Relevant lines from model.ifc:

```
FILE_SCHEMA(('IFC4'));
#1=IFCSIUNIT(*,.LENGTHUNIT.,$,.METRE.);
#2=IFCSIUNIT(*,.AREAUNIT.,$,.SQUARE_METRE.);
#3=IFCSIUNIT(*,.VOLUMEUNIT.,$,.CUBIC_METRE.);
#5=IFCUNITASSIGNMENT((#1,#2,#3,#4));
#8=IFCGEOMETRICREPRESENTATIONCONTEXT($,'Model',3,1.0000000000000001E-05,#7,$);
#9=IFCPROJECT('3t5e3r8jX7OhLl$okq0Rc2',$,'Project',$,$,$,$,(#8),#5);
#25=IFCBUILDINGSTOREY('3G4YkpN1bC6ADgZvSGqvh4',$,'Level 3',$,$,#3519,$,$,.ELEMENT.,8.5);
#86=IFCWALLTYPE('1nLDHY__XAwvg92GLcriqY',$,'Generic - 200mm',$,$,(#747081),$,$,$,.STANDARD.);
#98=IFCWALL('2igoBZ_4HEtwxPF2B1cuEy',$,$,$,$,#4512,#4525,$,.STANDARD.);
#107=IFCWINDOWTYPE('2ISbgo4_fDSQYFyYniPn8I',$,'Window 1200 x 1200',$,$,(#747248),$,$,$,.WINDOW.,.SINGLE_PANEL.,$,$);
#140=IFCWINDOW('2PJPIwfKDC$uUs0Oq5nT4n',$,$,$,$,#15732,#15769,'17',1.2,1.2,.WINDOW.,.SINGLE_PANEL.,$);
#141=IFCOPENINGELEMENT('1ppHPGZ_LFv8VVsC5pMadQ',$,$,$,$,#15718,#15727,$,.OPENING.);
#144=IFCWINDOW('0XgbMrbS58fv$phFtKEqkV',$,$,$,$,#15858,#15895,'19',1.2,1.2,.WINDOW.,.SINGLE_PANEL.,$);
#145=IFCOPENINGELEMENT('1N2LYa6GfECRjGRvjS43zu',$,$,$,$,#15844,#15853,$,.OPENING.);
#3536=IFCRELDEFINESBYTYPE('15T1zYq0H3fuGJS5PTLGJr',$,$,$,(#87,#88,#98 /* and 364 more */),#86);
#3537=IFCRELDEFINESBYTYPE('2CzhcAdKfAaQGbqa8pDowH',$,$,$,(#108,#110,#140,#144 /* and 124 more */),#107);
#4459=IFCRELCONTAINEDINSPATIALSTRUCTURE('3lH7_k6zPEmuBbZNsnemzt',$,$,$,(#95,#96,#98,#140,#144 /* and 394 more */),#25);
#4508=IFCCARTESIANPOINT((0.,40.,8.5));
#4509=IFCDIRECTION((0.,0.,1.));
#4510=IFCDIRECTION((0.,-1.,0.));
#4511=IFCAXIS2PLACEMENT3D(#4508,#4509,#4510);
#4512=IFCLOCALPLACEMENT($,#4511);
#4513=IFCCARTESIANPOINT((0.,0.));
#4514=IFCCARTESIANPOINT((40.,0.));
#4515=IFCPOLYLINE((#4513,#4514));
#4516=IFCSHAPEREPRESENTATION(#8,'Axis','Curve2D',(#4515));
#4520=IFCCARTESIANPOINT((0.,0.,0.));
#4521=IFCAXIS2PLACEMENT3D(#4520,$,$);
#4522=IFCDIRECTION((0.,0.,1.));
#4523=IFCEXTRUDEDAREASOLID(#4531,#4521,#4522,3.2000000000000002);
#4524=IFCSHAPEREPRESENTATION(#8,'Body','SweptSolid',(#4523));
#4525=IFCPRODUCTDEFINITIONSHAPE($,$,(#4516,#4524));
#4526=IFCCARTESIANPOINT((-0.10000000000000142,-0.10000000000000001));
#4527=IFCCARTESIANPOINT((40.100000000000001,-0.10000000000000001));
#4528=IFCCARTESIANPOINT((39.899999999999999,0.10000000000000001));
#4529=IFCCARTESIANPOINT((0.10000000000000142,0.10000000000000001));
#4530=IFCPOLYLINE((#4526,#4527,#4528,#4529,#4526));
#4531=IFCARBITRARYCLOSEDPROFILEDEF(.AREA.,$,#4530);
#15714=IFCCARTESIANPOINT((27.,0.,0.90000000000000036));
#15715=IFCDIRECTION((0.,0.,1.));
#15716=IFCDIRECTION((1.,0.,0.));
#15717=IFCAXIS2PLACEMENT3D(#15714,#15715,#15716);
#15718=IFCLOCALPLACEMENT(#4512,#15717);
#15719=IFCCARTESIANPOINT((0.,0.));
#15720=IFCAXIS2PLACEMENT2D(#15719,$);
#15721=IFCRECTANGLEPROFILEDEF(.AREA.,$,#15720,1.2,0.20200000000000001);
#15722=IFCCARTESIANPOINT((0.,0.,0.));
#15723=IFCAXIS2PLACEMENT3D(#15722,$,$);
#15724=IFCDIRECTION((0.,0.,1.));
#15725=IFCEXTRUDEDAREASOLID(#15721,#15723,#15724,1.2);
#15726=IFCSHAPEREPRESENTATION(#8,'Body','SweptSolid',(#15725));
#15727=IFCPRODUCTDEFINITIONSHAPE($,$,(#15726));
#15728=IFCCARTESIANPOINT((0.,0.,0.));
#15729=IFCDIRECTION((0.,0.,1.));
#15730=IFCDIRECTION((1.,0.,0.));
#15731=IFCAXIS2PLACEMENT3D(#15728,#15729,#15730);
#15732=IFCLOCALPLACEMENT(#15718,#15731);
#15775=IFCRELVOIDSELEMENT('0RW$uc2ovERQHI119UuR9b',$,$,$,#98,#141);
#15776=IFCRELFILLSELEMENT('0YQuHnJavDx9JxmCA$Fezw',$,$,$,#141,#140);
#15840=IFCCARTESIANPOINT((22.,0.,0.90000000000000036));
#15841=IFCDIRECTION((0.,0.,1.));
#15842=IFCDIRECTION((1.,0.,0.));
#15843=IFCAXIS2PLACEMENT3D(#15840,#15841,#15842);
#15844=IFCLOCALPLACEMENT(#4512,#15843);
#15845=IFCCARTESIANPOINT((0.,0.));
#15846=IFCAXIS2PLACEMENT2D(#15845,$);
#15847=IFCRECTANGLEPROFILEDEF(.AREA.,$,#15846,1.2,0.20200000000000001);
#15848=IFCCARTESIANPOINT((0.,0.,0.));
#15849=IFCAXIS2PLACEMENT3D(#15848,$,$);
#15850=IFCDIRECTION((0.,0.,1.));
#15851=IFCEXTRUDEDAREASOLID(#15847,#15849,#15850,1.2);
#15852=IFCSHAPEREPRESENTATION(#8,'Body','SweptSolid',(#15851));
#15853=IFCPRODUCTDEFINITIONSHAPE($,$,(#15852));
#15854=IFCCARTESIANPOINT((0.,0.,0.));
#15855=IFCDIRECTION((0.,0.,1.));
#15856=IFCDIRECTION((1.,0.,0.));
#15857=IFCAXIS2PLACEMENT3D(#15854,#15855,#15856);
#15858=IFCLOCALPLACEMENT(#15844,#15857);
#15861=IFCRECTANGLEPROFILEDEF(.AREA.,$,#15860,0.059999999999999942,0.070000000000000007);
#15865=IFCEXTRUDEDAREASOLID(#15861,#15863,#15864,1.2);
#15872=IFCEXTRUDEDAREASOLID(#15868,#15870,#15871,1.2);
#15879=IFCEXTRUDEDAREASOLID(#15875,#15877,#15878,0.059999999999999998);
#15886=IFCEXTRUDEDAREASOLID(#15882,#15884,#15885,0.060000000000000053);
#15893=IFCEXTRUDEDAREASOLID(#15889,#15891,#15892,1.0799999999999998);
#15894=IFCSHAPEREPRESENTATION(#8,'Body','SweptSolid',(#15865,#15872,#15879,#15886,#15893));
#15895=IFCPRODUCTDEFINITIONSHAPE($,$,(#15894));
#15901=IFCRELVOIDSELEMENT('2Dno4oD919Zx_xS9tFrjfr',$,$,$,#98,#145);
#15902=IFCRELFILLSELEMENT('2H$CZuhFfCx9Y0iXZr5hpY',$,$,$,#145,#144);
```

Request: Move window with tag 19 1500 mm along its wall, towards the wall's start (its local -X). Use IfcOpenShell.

```python
import ifcopenshell
import ifcopenshell.api.geometry
import ifcopenshell.util.placement
import ifcopenshell.util.unit

model = ifcopenshell.open("model.ifc")
unit_scale = ifcopenshell.util.unit.calculate_unit_scale(model)

window = model.by_id(144)
opening = window.FillsVoids[0].RelatingOpeningElement
wall = opening.VoidsElements[0].RelatingBuildingElement

wall_matrix = ifcopenshell.util.placement.get_local_placement(wall.ObjectPlacement)
shift = wall_matrix[:3, 0] * -1.5 / unit_scale
before = ifcopenshell.util.placement.get_local_placement(window.ObjectPlacement)[:3, 3].copy()

# The window is placed relative to its opening, so it follows when the opening moves.
matrix = ifcopenshell.util.placement.get_local_placement(opening.ObjectPlacement)
matrix[:3, 3] += shift
ifcopenshell.api.geometry.edit_object_placement(
    model, product=opening, matrix=matrix, is_si=False, should_transform_children=True
)

after = ifcopenshell.util.placement.get_local_placement(window.ObjectPlacement)[:3, 3]
print("window moved by", (after - before).round(3) + 0.0)

model.write("model_rev.ifc")
```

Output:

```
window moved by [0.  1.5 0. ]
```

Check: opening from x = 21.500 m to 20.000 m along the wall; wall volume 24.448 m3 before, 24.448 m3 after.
